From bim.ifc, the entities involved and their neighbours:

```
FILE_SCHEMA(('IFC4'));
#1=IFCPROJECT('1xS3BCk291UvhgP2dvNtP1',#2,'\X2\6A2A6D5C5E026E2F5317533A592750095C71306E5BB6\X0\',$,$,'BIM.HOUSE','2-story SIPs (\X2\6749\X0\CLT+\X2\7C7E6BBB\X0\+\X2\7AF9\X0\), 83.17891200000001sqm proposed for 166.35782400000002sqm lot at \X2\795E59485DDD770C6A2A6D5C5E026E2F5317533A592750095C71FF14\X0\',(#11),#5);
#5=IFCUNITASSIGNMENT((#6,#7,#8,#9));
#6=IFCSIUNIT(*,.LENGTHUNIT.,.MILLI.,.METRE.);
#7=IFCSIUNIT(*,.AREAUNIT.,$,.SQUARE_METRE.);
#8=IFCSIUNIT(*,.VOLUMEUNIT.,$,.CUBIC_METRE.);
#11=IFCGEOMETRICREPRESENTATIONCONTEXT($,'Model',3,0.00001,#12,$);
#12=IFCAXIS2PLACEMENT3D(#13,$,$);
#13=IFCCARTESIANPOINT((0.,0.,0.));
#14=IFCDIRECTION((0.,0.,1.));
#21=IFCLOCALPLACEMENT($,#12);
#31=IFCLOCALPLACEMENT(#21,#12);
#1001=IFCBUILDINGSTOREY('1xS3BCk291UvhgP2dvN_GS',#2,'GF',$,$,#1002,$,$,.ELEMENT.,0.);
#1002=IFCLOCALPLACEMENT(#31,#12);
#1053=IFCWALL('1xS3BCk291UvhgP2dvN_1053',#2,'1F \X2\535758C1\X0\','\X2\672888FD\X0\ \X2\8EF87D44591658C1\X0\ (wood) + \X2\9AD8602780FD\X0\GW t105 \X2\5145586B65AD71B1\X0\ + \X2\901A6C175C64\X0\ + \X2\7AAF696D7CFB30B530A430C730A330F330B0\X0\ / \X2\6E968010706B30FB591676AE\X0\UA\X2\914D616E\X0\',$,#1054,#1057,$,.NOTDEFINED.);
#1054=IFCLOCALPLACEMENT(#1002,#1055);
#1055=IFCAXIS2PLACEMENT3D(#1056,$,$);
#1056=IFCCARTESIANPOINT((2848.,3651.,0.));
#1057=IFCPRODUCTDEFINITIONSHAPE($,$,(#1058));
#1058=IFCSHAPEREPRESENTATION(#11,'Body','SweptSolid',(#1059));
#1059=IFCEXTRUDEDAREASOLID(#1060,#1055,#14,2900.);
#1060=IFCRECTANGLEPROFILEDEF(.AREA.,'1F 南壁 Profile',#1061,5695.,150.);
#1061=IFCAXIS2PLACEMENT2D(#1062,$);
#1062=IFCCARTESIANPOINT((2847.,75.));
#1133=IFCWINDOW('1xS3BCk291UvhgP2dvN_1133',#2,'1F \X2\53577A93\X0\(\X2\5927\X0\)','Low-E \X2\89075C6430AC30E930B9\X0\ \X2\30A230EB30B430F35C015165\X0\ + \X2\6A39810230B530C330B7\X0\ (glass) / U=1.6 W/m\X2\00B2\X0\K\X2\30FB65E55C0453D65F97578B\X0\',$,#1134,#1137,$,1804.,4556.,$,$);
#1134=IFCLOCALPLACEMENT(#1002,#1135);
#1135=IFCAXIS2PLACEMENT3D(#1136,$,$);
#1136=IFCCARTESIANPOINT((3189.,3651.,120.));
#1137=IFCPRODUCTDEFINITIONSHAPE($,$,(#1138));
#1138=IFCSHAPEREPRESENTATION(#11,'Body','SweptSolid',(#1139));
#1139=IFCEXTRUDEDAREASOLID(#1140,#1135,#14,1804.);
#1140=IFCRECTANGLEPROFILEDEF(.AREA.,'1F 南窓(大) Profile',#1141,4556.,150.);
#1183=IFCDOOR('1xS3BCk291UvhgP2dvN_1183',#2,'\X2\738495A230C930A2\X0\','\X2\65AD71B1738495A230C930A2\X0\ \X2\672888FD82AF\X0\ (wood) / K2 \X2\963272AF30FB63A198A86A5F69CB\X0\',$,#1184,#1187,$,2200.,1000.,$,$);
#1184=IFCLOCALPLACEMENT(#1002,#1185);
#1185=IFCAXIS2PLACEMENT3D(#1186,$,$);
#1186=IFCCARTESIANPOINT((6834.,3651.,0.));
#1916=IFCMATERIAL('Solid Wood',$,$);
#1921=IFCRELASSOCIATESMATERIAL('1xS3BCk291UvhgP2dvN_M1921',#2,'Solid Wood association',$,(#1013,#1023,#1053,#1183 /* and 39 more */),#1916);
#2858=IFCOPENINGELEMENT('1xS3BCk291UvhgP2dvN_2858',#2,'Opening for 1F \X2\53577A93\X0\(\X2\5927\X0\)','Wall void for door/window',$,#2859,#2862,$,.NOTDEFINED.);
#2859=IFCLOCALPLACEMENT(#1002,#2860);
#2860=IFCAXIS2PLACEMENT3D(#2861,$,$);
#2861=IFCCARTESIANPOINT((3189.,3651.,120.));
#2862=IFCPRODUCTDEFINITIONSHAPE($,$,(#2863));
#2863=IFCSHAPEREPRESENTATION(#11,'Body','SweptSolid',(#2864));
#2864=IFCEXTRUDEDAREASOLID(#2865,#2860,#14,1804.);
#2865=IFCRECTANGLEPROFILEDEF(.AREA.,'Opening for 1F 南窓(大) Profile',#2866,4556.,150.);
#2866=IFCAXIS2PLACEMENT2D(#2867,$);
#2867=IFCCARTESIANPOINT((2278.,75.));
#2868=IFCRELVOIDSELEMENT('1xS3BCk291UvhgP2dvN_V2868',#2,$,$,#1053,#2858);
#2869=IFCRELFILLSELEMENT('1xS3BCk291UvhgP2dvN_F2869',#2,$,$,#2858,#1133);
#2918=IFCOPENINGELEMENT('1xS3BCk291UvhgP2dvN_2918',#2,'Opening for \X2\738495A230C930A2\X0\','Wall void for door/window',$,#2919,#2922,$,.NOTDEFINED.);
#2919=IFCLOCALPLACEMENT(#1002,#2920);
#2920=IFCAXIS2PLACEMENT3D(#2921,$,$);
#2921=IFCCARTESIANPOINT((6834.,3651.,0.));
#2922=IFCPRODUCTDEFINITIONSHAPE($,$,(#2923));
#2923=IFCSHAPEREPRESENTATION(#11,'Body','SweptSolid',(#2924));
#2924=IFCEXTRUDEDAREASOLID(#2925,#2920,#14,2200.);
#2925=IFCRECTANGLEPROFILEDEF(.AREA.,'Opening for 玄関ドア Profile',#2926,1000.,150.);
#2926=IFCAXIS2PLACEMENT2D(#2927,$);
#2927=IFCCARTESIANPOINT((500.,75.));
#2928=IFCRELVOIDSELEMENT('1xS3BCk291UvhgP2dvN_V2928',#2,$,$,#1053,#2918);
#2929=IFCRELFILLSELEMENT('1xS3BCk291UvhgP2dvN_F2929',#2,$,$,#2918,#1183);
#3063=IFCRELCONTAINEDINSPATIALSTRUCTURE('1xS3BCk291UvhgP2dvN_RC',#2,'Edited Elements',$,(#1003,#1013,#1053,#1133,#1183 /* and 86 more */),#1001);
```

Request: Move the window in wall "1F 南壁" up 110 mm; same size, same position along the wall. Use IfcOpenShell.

```python
import numpy as np
import ifcopenshell
import ifcopenshell.api.geometry
import ifcopenshell.util.placement
import ifcopenshell.util.unit

model = ifcopenshell.open("bim.ifc")
unit_scale = ifcopenshell.util.unit.calculate_unit_scale(model)

window = model.by_id(1133)
opening = window.FillsVoids[0].RelatingOpeningElement
dz = 0.11 / unit_scale

shift = np.array([0.0, 0.0, dz])
# The window is not placed relative to its opening, so move both.
for product in (opening, window):
    matrix = ifcopenshell.util.placement.get_local_placement(product.ObjectPlacement)
    matrix[:3, 3] += shift
    ifcopenshell.api.geometry.edit_object_placement(model, product=product, matrix=matrix, is_si=False)

print(f"moved by {dz * unit_scale:+.3f} m")

model.write("bim_edited.ifc")
```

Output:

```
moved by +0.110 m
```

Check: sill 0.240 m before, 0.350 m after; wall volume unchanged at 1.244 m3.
